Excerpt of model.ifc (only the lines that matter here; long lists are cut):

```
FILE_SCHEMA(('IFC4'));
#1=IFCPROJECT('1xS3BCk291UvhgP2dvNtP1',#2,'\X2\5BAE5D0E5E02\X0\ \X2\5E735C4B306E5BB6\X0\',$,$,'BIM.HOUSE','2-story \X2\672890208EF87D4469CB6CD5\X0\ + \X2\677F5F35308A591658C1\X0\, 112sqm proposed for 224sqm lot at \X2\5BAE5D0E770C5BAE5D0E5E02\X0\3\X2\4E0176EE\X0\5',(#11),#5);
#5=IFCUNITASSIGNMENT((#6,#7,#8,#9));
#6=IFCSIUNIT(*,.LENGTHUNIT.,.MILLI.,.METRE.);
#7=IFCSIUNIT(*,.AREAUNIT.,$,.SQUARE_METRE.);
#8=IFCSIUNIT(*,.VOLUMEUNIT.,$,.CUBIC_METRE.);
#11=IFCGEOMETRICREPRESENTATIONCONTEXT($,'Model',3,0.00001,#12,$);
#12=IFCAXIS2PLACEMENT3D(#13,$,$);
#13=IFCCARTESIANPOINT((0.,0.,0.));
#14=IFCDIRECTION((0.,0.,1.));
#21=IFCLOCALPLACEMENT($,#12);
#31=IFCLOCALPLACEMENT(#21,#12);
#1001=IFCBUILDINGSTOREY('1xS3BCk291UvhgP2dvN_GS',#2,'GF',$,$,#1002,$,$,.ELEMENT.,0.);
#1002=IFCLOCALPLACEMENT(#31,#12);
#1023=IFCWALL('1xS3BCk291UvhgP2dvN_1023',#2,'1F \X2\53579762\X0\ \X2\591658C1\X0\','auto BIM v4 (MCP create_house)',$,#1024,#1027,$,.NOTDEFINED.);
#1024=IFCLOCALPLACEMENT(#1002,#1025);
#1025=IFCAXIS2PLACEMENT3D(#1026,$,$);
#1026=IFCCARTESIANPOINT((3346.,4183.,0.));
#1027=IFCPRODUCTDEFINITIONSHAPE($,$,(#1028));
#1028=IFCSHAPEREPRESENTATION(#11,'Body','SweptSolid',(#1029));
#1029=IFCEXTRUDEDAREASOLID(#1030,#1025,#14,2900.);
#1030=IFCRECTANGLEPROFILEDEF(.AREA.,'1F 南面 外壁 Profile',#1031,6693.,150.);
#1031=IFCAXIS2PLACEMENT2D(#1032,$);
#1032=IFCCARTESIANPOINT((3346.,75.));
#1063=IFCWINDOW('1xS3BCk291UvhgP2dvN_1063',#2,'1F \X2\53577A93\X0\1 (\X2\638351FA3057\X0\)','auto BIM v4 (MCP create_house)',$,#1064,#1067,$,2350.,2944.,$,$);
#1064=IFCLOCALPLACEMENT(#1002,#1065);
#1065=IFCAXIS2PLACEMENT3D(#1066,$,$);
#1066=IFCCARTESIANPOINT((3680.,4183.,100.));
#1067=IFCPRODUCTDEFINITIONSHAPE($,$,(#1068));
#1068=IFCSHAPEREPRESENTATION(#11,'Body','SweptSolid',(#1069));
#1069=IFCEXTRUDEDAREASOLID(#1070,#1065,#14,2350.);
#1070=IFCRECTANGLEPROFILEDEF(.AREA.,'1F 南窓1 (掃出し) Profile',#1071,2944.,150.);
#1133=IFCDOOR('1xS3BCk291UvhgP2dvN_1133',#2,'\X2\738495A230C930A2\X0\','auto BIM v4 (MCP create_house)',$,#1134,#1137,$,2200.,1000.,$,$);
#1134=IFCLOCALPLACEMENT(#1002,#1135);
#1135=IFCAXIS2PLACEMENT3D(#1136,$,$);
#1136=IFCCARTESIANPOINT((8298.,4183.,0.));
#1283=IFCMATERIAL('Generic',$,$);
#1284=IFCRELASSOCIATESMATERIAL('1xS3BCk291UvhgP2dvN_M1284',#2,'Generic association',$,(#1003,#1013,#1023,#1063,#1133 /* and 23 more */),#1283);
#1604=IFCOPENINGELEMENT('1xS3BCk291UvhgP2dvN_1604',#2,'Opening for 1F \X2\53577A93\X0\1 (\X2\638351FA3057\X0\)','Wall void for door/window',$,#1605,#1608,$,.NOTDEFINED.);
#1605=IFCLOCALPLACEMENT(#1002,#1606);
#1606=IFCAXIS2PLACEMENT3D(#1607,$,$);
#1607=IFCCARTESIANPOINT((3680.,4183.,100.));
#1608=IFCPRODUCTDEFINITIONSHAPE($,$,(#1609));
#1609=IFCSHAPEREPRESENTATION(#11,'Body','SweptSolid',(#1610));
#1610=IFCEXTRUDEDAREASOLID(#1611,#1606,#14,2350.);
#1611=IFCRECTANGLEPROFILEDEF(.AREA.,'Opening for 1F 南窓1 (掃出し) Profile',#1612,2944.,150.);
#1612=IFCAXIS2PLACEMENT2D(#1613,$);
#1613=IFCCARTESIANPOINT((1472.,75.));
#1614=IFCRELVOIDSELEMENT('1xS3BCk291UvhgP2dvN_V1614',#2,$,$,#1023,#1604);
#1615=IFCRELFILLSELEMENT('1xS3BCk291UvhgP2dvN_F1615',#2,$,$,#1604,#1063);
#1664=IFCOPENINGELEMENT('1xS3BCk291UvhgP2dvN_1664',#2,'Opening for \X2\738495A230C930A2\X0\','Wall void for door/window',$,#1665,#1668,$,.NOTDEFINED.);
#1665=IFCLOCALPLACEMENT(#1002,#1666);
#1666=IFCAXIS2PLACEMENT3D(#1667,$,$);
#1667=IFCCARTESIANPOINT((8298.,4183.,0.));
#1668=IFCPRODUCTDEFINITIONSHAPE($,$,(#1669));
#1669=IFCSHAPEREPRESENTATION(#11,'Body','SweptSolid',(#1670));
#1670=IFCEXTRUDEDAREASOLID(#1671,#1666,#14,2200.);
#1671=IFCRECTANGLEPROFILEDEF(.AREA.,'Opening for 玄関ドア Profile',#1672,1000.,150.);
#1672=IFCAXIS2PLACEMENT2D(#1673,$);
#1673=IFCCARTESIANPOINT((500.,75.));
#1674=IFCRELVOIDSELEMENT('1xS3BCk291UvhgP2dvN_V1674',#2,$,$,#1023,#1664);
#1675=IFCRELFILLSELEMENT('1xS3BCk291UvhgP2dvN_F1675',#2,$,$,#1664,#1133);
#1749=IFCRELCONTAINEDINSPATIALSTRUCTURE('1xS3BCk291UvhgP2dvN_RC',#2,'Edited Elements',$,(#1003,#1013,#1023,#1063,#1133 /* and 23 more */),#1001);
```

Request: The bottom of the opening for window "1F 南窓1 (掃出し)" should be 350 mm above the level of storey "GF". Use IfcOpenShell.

```python
import numpy as np
import ifcopenshell
import ifcopenshell.api.geometry
import ifcopenshell.geom
import ifcopenshell.util.element
import ifcopenshell.util.placement
import ifcopenshell.util.shape
import ifcopenshell.util.unit

model = ifcopenshell.open("model.ifc")
unit_scale = ifcopenshell.util.unit.calculate_unit_scale(model)

window = model.by_guid("1xS3BCk291UvhgP2dvN_1063")
opening = window.FillsVoids[0].RelatingOpeningElement
storey = ifcopenshell.util.element.get_container(window, ifc_class="IfcBuildingStorey")
level = ifcopenshell.util.placement.get_local_placement(storey.ObjectPlacement)[2, 3]

# The opening's origin need not be at the sill, so measure its lowest point.
shape = ifcopenshell.geom.create_shape(ifcopenshell.geom.settings(), opening)
bottom = ifcopenshell.util.shape.get_shape_bottom_elevation(shape, shape.geometry) / unit_scale
dz = level + 350.0 - bottom

shift = np.array([0.0, 0.0, dz])
# The window is not placed relative to its opening, so move both.
for product in (opening, window):
    matrix = ifcopenshell.util.placement.get_local_placement(product.ObjectPlacement)
    matrix[:3, 3] += shift
    ifcopenshell.api.geometry.edit_object_placement(model, product=product, matrix=matrix, is_si=False)

print(f"moved by {dz * unit_scale:+.3f} m")

model.write("model_rev.ifc")
```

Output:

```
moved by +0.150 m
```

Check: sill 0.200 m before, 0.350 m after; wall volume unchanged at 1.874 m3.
